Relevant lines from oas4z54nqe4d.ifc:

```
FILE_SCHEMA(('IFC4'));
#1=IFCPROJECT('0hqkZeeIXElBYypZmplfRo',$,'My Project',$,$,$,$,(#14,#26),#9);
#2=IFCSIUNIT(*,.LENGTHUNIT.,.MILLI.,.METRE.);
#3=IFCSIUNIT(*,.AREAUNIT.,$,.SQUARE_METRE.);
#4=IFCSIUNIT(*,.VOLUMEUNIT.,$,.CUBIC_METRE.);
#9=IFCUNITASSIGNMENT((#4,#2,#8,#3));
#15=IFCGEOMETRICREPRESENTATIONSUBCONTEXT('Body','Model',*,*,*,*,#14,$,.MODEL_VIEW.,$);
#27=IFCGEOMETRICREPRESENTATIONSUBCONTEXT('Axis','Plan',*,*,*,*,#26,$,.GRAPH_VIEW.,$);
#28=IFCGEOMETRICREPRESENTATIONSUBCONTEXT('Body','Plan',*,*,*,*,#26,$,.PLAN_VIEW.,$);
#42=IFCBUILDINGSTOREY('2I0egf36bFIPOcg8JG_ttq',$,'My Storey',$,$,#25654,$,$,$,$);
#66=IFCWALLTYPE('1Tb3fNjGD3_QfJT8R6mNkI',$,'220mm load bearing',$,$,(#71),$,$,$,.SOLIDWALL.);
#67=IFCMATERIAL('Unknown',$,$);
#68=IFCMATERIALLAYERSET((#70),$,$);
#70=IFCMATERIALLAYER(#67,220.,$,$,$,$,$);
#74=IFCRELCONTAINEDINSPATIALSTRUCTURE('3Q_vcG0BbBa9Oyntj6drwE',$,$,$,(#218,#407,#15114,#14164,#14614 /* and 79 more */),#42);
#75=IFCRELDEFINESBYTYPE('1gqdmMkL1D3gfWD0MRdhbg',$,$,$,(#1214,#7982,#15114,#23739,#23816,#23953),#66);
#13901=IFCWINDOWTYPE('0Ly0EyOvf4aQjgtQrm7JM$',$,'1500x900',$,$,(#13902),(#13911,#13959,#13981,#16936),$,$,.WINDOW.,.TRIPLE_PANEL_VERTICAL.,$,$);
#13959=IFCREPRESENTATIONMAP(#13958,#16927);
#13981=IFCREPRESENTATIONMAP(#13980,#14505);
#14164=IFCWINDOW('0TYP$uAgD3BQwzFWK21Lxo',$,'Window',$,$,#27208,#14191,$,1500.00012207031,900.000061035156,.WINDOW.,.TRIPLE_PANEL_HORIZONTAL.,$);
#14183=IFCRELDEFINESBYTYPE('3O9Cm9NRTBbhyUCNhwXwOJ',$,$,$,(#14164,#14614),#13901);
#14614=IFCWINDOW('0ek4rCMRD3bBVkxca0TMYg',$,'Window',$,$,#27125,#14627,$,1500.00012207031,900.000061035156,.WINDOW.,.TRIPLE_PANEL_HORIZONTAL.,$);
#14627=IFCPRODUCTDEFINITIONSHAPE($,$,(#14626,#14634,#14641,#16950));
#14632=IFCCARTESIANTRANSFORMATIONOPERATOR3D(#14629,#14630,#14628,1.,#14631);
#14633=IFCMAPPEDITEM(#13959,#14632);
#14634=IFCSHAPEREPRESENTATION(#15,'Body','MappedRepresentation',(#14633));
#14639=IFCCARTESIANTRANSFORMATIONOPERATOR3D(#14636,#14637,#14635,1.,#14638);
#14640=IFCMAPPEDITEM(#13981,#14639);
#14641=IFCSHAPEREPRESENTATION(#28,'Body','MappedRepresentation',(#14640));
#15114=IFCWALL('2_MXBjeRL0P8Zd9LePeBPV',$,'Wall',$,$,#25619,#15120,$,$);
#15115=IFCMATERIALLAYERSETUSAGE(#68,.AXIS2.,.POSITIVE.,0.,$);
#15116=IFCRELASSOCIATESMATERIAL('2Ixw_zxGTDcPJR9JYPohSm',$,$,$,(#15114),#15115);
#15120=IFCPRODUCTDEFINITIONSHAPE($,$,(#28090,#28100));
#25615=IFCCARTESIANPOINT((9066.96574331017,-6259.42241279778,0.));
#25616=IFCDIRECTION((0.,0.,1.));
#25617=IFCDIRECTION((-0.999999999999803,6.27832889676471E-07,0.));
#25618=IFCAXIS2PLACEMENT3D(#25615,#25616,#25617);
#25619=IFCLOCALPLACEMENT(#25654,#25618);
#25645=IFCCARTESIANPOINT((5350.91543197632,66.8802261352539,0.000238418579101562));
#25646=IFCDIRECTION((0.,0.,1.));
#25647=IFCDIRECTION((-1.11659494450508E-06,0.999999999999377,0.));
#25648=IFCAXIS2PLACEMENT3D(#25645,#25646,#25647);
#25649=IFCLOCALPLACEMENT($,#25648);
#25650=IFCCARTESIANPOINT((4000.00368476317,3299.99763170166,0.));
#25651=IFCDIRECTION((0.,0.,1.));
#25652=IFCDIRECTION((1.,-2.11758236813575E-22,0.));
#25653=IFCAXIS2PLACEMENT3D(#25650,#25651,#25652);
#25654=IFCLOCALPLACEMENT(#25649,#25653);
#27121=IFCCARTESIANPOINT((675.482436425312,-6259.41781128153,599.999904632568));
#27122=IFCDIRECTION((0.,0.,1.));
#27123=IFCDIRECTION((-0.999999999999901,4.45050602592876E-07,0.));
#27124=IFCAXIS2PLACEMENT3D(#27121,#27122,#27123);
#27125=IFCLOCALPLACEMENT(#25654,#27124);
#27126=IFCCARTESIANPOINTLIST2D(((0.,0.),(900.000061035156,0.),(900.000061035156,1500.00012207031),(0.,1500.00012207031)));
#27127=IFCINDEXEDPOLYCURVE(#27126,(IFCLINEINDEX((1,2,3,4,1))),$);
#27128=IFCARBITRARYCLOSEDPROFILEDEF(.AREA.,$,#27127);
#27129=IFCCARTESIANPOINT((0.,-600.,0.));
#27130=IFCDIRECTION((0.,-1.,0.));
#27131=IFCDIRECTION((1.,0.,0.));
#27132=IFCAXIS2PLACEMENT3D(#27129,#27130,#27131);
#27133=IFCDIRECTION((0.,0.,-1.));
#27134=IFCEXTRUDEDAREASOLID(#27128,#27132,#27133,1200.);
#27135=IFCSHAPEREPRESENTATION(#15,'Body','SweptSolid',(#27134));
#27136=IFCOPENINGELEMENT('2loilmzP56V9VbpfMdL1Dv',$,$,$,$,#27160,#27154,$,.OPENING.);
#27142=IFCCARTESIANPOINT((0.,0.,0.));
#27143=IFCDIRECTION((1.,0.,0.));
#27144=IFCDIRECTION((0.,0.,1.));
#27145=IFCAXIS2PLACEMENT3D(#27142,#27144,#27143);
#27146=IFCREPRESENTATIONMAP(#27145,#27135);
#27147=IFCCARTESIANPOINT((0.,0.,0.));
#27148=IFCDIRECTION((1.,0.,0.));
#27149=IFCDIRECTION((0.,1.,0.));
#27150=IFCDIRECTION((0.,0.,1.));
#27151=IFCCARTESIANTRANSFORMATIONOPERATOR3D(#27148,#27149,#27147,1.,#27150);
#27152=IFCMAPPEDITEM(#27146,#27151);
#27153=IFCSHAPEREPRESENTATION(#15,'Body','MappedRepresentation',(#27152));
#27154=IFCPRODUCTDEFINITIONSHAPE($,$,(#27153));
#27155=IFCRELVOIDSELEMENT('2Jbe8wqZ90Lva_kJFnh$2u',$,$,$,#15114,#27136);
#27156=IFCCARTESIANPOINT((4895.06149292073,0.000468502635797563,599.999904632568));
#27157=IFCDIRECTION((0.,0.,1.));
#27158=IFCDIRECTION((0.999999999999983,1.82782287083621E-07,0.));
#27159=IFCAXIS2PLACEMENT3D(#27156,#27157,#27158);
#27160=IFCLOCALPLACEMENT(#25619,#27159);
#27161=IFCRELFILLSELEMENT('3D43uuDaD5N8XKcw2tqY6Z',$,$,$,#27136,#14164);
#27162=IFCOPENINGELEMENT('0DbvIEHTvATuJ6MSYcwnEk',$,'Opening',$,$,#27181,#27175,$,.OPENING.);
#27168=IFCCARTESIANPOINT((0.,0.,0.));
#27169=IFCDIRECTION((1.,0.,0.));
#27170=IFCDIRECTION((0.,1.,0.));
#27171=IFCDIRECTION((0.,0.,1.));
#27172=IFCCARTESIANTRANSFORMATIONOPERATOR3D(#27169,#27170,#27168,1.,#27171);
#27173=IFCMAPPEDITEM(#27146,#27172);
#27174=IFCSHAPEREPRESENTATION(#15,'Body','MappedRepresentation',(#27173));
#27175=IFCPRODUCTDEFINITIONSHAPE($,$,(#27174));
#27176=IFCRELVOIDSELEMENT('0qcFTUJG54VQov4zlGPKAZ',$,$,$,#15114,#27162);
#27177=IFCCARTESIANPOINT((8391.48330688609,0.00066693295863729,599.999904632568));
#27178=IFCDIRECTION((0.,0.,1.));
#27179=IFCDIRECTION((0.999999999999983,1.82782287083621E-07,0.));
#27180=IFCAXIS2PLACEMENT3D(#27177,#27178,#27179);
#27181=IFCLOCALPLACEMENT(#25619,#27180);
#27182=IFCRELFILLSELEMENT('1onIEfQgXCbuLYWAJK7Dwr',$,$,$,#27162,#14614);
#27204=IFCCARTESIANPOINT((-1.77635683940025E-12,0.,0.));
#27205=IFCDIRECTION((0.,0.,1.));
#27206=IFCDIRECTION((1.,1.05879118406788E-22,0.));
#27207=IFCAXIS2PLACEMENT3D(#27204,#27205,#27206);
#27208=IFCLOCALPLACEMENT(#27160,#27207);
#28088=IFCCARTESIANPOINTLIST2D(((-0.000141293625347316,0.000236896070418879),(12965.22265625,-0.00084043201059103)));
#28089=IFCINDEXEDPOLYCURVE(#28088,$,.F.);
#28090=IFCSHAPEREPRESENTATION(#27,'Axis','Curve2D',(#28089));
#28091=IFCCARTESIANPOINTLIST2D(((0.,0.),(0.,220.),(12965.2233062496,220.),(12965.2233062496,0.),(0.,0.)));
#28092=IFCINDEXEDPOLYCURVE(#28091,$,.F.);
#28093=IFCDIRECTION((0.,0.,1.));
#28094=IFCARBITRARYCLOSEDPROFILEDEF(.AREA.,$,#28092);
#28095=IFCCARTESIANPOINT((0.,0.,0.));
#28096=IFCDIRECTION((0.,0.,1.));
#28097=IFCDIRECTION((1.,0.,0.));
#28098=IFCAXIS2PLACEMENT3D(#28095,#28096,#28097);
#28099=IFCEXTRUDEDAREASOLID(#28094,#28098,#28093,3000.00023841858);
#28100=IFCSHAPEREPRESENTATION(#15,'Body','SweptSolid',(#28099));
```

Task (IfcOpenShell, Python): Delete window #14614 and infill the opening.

```python
import ifcopenshell
import ifcopenshell.api.feature
import ifcopenshell.api.root
import ifcopenshell.geom
import ifcopenshell.util.shape

model = ifcopenshell.open("oas4z54nqe4d.ifc")
settings = ifcopenshell.geom.settings()


def volume(element):
    """Net volume in cubic metres, openings subtracted."""
    shape = ifcopenshell.geom.create_shape(settings, element)
    return ifcopenshell.util.shape.get_volume(shape.geometry)


window = model.by_id(14614)
opening = window.FillsVoids[0].RelatingOpeningElement
wall = opening.VoidsElements[0].RelatingBuildingElement
before = volume(wall)

ifcopenshell.api.root.remove_product(model, product=window)
ifcopenshell.api.feature.remove_feature(model, feature=opening)

after = volume(wall)

print(f"wall volume {before:.3f} -> {after:.3f} m3")

model.write("oas4z54nqe4d-out.ifc")
```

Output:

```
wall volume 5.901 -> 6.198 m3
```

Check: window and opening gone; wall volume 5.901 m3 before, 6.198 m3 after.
